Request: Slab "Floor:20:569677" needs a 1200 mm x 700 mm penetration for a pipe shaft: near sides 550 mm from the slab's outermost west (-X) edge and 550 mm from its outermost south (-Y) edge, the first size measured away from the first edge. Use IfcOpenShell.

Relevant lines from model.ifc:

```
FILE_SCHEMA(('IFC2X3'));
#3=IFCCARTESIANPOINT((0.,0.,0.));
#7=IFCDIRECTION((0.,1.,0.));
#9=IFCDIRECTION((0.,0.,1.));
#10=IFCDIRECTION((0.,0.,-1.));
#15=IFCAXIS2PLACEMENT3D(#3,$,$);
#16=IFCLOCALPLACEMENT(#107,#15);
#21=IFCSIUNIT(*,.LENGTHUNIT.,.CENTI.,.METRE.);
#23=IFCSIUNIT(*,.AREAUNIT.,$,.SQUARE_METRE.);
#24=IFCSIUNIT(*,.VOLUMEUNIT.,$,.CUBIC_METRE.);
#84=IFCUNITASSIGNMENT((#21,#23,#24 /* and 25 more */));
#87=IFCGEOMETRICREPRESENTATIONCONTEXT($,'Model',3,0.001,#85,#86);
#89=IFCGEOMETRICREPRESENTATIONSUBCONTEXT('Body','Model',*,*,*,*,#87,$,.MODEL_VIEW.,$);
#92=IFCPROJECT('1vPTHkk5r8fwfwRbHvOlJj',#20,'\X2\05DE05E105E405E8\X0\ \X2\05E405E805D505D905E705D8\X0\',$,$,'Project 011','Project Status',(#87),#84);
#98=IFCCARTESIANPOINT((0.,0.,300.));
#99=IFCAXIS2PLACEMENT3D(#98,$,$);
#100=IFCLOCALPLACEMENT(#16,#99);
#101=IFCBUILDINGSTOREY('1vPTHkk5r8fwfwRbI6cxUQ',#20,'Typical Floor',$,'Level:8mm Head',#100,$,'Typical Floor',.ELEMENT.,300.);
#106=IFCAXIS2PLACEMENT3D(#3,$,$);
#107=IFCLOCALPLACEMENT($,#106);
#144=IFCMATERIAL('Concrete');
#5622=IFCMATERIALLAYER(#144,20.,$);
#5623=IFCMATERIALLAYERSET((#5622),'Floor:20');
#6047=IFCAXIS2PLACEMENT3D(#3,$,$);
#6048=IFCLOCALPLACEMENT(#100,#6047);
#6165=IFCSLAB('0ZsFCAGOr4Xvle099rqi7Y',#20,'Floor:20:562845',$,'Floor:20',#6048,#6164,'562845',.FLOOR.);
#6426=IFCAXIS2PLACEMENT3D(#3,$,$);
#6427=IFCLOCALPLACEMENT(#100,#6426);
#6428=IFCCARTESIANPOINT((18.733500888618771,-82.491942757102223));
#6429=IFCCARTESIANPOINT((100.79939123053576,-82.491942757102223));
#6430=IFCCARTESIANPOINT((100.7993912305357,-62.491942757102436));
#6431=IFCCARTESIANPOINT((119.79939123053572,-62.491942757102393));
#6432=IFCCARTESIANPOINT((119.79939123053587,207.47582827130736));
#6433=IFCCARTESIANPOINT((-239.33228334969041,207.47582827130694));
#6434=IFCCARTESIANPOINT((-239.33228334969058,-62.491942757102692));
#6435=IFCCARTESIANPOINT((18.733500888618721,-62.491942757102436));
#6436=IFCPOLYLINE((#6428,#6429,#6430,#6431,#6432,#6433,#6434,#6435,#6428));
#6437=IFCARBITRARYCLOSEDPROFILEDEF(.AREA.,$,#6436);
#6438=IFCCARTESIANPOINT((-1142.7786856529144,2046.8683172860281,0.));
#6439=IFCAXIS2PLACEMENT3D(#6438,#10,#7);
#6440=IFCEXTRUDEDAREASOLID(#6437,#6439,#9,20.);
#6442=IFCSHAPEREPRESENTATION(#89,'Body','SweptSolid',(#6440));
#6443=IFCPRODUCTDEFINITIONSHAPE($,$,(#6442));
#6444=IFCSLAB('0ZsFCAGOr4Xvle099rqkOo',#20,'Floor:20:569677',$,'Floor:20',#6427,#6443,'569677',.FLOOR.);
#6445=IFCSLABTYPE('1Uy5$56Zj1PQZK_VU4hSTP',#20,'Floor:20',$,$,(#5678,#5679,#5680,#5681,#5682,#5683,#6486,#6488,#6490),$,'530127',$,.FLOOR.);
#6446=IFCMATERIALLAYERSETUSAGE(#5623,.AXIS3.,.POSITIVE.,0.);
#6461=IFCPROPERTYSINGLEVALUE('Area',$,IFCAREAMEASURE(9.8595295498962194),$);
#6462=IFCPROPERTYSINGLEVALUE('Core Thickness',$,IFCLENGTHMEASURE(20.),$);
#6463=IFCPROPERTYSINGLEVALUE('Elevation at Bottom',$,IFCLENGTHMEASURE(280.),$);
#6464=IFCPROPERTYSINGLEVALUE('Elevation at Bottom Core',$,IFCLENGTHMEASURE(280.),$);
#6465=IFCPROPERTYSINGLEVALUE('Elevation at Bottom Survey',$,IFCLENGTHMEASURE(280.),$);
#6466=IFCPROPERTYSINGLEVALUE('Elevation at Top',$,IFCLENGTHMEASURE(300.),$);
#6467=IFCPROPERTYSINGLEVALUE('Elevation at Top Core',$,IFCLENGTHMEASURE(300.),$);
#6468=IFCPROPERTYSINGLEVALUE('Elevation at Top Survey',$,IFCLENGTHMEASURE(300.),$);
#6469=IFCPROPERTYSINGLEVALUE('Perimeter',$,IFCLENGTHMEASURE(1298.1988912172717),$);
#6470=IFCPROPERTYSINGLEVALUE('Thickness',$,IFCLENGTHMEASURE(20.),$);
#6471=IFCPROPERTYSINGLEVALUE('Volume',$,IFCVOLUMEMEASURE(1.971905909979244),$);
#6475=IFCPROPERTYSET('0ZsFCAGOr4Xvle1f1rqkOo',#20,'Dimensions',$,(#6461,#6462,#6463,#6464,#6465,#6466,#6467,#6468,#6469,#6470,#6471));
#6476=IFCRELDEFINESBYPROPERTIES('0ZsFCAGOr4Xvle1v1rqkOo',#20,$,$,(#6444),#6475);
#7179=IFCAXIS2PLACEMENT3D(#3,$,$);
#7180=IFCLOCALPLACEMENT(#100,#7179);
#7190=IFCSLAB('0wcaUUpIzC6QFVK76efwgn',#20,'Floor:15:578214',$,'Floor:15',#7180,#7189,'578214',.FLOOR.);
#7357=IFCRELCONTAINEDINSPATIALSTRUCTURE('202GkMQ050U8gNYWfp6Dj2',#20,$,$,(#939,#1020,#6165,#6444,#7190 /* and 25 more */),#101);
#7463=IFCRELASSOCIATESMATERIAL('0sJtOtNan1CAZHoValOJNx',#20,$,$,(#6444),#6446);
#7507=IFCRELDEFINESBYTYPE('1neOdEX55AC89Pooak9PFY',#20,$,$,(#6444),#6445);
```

```python
import numpy as np
import ifcopenshell
import ifcopenshell.api.feature
import ifcopenshell.api.geometry
import ifcopenshell.api.pset
import ifcopenshell.api.root
import ifcopenshell.geom
import ifcopenshell.util.element
import ifcopenshell.util.placement
import ifcopenshell.util.representation
import ifcopenshell.util.shape
import ifcopenshell.util.unit

model = ifcopenshell.open("model.ifc")
unit_scale = ifcopenshell.util.unit.calculate_unit_scale(model)
area_scale = ifcopenshell.util.unit.calculate_unit_scale(model, "AREAUNIT")
volume_scale = ifcopenshell.util.unit.calculate_unit_scale(model, "VOLUMEUNIT")
settings = ifcopenshell.geom.settings()


def volume(element):
    """Net volume in cubic metres, openings subtracted."""
    shape = ifcopenshell.geom.create_shape(settings, element)
    return ifcopenshell.util.shape.get_volume(shape.geometry)


slab = model.by_guid("0ZsFCAGOr4Xvle099rqkOo")
before = volume(slab)

# Extent in the slab's own axes, in metres. The edges named are its -X and -Y sides.
slab_shape = ifcopenshell.geom.create_shape(settings, slab)
vertices = ifcopenshell.util.shape.get_vertices(slab_shape.geometry)
x_min, y_min, bottom = vertices.min(axis=0)
top = vertices[:, 2].max()

opening = ifcopenshell.api.root.create_entity(model, ifc_class="IfcOpeningElement", name="Pipe shaft opening")
context = ifcopenshell.util.representation.get_context(model, "Model", "Body", "MODEL_VIEW")
width, depth = 1.2, 0.7
outline = [(0.0, 0.0), (width, 0.0), (width, depth), (0.0, depth), (0.0, 0.0)]
# Overshoot both faces by 50 mm so the cut is clean.
shape = ifcopenshell.api.geometry.add_slab_representation(
    model, context=context, depth=top - bottom + 0.1, polyline=outline
)
ifcopenshell.api.geometry.assign_representation(model, product=opening, representation=shape)

matrix = ifcopenshell.util.placement.get_local_placement(slab.ObjectPlacement)
matrix[:, 3] = matrix @ np.append(np.array([x_min + 0.55, y_min + 0.55, bottom - 0.05]) / unit_scale, 1.0)
ifcopenshell.api.geometry.edit_object_placement(model, product=opening, matrix=matrix, is_si=False)
ifcopenshell.api.feature.add_feature(model, feature=opening, element=slab)

after = volume(slab)

# Update the slab's stored quantities.
pset = model.by_id(ifcopenshell.util.element.get_pset(slab, "Dimensions", should_inherit=False)["id"])
ifcopenshell.api.pset.edit_pset(model, pset=pset, properties={
    "Area": model.create_entity("IfcAreaMeasure", after / (top - bottom) / area_scale),
    "Volume": model.create_entity("IfcVolumeMeasure", after / volume_scale),
})

print(f"slab volume {before:.3f} -> {after:.3f} m3")

model.write("model_rev.ifc")
```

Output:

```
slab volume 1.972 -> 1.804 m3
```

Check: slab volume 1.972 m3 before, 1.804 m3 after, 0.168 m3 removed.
